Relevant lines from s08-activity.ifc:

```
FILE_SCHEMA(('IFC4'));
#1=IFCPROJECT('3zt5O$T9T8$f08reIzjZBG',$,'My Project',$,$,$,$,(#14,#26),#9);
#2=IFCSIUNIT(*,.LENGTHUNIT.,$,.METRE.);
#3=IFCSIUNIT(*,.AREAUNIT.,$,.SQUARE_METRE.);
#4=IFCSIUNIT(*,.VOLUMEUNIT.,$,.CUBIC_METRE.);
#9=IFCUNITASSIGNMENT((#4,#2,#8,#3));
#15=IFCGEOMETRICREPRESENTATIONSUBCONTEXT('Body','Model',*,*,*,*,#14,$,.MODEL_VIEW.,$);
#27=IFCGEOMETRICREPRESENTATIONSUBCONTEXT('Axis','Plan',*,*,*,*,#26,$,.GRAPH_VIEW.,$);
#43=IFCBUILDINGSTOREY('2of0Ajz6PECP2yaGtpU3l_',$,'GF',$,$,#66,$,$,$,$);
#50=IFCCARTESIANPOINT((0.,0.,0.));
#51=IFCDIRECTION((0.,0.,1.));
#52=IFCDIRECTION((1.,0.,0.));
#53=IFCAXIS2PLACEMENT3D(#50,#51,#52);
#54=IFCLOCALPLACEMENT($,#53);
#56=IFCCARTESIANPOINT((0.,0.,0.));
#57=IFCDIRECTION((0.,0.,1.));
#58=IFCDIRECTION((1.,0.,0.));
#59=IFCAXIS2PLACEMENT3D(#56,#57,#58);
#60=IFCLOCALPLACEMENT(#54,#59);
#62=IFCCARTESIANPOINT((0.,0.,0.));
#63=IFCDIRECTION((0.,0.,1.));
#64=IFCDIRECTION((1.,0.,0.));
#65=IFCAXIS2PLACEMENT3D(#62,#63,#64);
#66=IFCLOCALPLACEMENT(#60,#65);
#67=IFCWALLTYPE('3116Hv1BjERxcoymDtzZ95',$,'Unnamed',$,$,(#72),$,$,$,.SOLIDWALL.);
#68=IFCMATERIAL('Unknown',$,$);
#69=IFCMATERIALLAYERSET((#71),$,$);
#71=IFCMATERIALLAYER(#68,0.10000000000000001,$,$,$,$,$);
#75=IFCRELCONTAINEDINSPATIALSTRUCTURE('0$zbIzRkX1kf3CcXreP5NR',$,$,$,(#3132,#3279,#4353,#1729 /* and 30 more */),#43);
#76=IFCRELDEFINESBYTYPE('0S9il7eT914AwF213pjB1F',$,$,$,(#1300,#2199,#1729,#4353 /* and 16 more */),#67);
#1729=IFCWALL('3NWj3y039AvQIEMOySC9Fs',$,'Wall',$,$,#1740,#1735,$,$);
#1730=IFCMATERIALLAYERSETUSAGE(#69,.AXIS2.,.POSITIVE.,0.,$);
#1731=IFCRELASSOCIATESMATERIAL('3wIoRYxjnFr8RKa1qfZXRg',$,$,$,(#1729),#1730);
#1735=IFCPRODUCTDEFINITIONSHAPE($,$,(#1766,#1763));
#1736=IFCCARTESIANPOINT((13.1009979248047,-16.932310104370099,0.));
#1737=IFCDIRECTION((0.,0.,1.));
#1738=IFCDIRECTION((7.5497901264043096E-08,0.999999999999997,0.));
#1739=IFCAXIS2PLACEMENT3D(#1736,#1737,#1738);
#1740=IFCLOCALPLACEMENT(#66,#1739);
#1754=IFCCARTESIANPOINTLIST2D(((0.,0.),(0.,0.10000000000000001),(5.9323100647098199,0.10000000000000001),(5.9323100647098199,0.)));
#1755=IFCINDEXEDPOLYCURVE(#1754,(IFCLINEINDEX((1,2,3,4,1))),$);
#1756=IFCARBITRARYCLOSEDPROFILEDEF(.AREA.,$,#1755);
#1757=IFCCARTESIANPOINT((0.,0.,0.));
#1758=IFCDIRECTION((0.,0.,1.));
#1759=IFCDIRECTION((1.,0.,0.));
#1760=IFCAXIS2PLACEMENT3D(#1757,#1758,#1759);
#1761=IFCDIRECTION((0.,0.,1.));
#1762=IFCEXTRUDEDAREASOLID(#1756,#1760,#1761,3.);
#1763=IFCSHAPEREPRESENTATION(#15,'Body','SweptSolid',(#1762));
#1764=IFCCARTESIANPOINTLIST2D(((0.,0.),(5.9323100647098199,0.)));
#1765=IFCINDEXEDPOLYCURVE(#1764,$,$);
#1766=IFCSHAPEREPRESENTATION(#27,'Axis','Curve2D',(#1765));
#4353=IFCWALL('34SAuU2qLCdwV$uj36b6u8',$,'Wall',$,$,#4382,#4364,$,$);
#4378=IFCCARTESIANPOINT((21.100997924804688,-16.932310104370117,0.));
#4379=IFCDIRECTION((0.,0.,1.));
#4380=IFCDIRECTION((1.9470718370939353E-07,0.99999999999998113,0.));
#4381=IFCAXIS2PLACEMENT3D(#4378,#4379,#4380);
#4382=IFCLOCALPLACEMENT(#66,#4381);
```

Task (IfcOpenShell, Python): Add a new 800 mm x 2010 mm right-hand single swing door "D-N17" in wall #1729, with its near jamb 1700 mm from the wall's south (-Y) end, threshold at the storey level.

```python
import numpy as np
import ifcopenshell
import ifcopenshell.api.feature
import ifcopenshell.api.geometry
import ifcopenshell.api.root
import ifcopenshell.api.spatial
import ifcopenshell.geom
import ifcopenshell.util.element
import ifcopenshell.util.placement
import ifcopenshell.util.representation
import ifcopenshell.util.shape
import ifcopenshell.util.unit

model = ifcopenshell.open("s08-activity.ifc")
unit_scale = ifcopenshell.util.unit.calculate_unit_scale(model)
settings = ifcopenshell.geom.settings()


def volume(element):
    """Net volume in cubic metres, openings subtracted."""
    shape = ifcopenshell.geom.create_shape(settings, element)
    return ifcopenshell.util.shape.get_volume(shape.geometry)


wall = model.by_guid("3NWj3y039AvQIEMOySC9Fs")
storey = ifcopenshell.util.element.get_container(wall, ifc_class="IfcBuildingStorey")
context = ifcopenshell.util.representation.get_context(model, "Model", "Body", "MODEL_VIEW")
before = volume(wall)

width, height, from_end, sill = 0.8, 2.01, 1.7, 0.0  # metres

# The wall runs along its own X axis, and the end named is its -X end.
wall_shape = ifcopenshell.geom.create_shape(settings, wall)
x, y, z = ifcopenshell.util.shape.get_vertices(wall_shape.geometry).T
start = x.min() + from_end
face, thickness = float(y.min()), float(y.max() - y.min())
wall_matrix = ifcopenshell.util.placement.get_local_placement(wall.ObjectPlacement)
level = ifcopenshell.util.placement.get_local_placement(storey.ObjectPlacement)[2, 3]


def in_wall(x, y):
    """Placement at x, y metres in the wall's axes, at sill height."""
    matrix = wall_matrix.copy()
    matrix[:, 3] = wall_matrix @ np.array([x / unit_scale, y / unit_scale, 0.0, 1.0])
    matrix[2, 3] = level + sill / unit_scale
    return matrix


# Opening: a box that overshoots both wall faces by 50 mm.
opening = ifcopenshell.api.root.create_entity(model, ifc_class="IfcOpeningElement", predefined_type="OPENING")
box = ifcopenshell.api.geometry.add_wall_representation(
    model, context=context, length=width, height=height, thickness=thickness + 0.1
)
ifcopenshell.api.geometry.assign_representation(model, product=opening, representation=box)
ifcopenshell.api.geometry.edit_object_placement(model, product=opening, matrix=in_wall(start, face - 0.05), is_si=False)
ifcopenshell.api.feature.add_feature(model, feature=opening, element=wall)

door = ifcopenshell.api.root.create_entity(model, ifc_class="IfcDoor", name="D-N17", predefined_type="DOOR")
door.OverallWidth, door.OverallHeight = width / unit_scale, height / unit_scale
door.OperationType = "SINGLE_SWING_RIGHT"
body = ifcopenshell.api.geometry.add_door_representation(
    model,
    context=context,
    overall_width=door.OverallWidth,
    overall_height=door.OverallHeight,
    operation_type="SINGLE_SWING_RIGHT",
    lining_properties={"LiningDepth": thickness / unit_scale, "ThresholdDepth": thickness / unit_scale},
)
ifcopenshell.api.geometry.assign_representation(model, product=door, representation=body)
ifcopenshell.api.spatial.assign_container(model, products=[door], relating_structure=storey)
ifcopenshell.api.feature.add_filling(model, opening=opening, element=door)

# The lining spans the wall, so the door starts at the wall face.
ifcopenshell.api.geometry.edit_object_placement(model, product=door, matrix=in_wall(start, face), is_si=False)

after = volume(wall)

print(f"wall volume {before:.3f} -> {after:.3f} m3")

model.write("s08-activity_edited.ifc")
```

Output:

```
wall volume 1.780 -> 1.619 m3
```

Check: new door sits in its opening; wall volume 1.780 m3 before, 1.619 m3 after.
